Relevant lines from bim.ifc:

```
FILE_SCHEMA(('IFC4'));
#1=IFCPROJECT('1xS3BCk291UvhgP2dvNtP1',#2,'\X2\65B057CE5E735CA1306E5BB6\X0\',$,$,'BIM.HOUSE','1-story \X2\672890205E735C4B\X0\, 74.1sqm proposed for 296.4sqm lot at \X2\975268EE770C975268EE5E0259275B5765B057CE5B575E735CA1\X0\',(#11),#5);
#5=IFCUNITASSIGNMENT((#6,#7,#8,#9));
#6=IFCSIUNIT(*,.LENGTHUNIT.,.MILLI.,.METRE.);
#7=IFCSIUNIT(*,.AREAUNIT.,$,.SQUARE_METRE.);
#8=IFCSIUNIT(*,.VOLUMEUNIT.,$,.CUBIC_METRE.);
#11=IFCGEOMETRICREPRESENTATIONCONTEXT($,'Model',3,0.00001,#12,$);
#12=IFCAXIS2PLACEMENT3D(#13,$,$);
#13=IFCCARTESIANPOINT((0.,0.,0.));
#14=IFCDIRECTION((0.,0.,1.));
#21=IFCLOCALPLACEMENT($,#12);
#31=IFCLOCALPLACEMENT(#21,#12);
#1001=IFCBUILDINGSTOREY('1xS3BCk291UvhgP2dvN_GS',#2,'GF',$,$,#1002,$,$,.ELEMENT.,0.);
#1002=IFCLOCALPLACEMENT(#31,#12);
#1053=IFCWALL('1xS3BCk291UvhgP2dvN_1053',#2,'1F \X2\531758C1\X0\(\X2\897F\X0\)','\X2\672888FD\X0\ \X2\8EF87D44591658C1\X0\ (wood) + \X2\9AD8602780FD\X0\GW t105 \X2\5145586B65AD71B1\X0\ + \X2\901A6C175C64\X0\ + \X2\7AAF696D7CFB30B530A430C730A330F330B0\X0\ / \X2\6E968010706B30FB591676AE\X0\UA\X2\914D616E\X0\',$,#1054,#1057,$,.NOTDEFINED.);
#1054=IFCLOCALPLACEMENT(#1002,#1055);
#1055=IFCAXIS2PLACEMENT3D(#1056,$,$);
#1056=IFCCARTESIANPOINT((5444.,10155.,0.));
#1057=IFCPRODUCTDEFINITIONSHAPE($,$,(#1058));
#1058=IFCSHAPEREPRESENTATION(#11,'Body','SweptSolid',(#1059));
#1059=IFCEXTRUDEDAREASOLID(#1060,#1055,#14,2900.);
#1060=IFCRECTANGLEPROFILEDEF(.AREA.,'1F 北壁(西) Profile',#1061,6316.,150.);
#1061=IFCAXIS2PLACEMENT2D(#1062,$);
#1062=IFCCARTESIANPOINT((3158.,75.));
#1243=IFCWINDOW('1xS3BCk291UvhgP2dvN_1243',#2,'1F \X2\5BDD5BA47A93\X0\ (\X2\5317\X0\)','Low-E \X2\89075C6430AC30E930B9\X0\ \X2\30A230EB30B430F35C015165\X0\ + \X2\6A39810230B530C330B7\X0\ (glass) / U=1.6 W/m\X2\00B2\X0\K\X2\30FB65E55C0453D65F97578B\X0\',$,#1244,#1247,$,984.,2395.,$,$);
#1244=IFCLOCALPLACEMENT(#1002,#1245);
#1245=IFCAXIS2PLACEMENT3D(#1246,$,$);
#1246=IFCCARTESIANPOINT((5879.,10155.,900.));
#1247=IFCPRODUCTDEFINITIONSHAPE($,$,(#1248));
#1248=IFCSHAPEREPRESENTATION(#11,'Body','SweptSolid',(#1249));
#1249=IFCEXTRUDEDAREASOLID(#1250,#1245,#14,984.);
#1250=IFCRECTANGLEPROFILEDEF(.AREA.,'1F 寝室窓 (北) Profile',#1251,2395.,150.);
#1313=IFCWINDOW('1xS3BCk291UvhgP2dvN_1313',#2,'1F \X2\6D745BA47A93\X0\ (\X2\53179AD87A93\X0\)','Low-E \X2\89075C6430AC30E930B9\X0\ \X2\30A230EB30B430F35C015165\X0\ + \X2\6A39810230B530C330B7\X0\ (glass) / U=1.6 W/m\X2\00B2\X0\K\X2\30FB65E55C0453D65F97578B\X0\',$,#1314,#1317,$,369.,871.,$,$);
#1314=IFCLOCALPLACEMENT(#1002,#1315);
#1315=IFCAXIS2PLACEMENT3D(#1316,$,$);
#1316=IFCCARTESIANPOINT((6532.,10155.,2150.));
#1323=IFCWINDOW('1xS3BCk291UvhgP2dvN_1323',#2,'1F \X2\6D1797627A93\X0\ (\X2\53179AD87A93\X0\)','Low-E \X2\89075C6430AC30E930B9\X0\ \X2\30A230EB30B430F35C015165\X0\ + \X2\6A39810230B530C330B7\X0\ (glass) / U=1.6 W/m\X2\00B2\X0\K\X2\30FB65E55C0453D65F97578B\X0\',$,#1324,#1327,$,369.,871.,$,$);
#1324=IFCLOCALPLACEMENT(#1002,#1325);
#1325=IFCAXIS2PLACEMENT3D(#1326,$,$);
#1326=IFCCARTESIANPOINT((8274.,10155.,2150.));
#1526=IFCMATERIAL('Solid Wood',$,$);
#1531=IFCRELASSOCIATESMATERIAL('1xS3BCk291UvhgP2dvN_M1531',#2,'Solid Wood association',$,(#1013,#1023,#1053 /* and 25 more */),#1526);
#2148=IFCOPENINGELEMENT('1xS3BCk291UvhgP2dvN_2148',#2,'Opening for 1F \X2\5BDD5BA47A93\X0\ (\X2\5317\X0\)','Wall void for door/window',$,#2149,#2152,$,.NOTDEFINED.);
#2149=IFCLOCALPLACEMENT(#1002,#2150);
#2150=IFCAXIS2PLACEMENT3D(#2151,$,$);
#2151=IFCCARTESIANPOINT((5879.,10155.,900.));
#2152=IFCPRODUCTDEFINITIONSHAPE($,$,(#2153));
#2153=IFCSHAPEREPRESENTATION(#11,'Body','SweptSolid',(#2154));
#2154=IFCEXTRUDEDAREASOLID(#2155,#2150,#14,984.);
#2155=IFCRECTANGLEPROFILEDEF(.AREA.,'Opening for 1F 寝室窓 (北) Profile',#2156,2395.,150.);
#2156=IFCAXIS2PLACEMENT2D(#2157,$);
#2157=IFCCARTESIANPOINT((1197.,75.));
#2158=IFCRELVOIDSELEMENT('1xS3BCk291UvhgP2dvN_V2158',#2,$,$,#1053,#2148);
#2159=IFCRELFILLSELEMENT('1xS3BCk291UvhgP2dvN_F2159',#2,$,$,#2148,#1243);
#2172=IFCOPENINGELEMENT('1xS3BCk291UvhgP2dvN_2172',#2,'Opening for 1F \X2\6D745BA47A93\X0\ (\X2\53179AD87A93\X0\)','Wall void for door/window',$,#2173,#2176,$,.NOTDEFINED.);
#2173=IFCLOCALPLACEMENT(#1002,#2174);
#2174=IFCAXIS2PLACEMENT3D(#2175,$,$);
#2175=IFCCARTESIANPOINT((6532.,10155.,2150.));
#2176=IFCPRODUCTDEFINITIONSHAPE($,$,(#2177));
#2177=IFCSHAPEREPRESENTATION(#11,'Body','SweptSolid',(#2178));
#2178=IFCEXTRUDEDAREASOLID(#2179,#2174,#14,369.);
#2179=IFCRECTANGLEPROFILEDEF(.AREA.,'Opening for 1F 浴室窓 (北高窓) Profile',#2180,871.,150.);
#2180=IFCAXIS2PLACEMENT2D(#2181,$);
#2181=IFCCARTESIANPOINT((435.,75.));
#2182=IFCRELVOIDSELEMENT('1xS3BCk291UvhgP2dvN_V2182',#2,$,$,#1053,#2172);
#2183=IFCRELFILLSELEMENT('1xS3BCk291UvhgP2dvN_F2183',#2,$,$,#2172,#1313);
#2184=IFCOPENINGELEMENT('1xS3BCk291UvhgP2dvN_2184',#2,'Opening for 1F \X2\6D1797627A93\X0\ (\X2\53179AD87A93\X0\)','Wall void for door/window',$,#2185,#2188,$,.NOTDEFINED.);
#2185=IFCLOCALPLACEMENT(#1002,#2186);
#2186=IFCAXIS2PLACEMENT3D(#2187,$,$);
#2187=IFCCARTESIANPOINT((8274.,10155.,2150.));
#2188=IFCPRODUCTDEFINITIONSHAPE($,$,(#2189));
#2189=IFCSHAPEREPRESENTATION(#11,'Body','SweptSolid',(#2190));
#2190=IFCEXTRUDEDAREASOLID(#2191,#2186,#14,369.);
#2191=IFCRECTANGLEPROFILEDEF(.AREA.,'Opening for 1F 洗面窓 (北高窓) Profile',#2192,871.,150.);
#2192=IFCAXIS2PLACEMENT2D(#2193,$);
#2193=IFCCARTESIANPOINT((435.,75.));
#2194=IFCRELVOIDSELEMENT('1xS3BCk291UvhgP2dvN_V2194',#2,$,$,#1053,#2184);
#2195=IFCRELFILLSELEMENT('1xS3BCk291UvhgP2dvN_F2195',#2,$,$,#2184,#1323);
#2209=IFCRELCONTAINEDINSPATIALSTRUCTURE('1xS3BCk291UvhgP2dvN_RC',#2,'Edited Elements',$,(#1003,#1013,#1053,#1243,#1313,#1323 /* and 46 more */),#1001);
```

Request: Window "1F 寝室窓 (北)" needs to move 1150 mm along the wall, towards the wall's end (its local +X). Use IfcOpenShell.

```python
import ifcopenshell
import ifcopenshell.api.geometry
import ifcopenshell.util.placement
import ifcopenshell.util.unit

model = ifcopenshell.open("bim.ifc")
unit_scale = ifcopenshell.util.unit.calculate_unit_scale(model)

window = model.by_guid("1xS3BCk291UvhgP2dvN_1243")
opening = window.FillsVoids[0].RelatingOpeningElement
wall = opening.VoidsElements[0].RelatingBuildingElement

wall_matrix = ifcopenshell.util.placement.get_local_placement(wall.ObjectPlacement)
shift = wall_matrix[:3, 0] * 1.15 / unit_scale
before = ifcopenshell.util.placement.get_local_placement(window.ObjectPlacement)[:3, 3].copy()

# The window is not placed relative to its opening, so move both.
for product in (opening, window):
    matrix = ifcopenshell.util.placement.get_local_placement(product.ObjectPlacement)
    matrix[:3, 3] += shift
    ifcopenshell.api.geometry.edit_object_placement(model, product=product, matrix=matrix, is_si=False)

after = ifcopenshell.util.placement.get_local_placement(window.ObjectPlacement)[:3, 3]
print("window moved by", (after - before).round(3) + 0.0)

model.write("bim_edited.ifc")
```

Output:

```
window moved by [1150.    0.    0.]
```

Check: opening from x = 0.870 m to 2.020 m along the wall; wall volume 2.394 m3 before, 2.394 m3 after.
